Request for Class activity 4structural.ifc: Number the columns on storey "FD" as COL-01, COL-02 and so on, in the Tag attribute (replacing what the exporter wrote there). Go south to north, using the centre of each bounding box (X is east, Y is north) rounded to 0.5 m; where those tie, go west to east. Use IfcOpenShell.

First a look at what the model holds.

```python
import ifcopenshell
import ifcopenshell.util.element
import ifcopenshell.util.placement

model = ifcopenshell.open("Class activity 4structural.ifc")
print(model.schema)
storey = next(s for s in model.by_type("IfcBuildingStorey") if s.Name == "FD")
columns = [e for e in ifcopenshell.util.element.get_decomposition(storey) if e.is_a("IfcColumn")]
for e in sorted(columns, key=lambda e: e.id()):
    origin = ifcopenshell.util.placement.get_local_placement(e.ObjectPlacement)[:3, 3]
    print(e.id(), e.Tag, e.Name, origin.round(2) + 0.0, sep=" | ")
```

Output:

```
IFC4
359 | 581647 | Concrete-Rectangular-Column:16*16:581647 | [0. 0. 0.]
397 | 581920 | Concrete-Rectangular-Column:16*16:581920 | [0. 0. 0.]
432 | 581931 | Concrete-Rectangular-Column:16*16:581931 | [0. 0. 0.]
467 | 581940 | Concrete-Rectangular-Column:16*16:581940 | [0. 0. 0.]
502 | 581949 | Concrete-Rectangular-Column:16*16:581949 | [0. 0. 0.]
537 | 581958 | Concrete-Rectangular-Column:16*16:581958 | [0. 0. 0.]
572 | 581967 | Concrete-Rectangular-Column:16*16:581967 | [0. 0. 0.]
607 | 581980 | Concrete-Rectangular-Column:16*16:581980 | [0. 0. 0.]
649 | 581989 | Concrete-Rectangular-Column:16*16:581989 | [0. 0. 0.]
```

```python
import ifcopenshell
import ifcopenshell.geom
import ifcopenshell.util.element
import ifcopenshell.util.shape

model = ifcopenshell.open("Class activity 4structural.ifc")
settings = ifcopenshell.geom.settings()
settings.set("use-world-coords", True)


def centre(element):
    shape = ifcopenshell.geom.create_shape(settings, element)
    return ifcopenshell.util.shape.get_bbox_centroid(shape.geometry)


storey = next(s for s in model.by_type("IfcBuildingStorey") if s.Name == "FD")
columns = [e for e in ifcopenshell.util.element.get_decomposition(storey) if e.is_a("IfcColumn")]

# Insertion points can sit at a corner or the storey origin, so sort by the geometry (in metres).
centres = {e: centre(e) for e in columns}
columns.sort(key=lambda e: (round(centres[e][1] / 0.5), centres[e][0]))

for i, e in enumerate(columns, start=1):
    number = f"COL-{i:02d}"
    e.Tag = number
    print(e.id(), number)

model.write("Class activity 4structural_v2.ifc")
```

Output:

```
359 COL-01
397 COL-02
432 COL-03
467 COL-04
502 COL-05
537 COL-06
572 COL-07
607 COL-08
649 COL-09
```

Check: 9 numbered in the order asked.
